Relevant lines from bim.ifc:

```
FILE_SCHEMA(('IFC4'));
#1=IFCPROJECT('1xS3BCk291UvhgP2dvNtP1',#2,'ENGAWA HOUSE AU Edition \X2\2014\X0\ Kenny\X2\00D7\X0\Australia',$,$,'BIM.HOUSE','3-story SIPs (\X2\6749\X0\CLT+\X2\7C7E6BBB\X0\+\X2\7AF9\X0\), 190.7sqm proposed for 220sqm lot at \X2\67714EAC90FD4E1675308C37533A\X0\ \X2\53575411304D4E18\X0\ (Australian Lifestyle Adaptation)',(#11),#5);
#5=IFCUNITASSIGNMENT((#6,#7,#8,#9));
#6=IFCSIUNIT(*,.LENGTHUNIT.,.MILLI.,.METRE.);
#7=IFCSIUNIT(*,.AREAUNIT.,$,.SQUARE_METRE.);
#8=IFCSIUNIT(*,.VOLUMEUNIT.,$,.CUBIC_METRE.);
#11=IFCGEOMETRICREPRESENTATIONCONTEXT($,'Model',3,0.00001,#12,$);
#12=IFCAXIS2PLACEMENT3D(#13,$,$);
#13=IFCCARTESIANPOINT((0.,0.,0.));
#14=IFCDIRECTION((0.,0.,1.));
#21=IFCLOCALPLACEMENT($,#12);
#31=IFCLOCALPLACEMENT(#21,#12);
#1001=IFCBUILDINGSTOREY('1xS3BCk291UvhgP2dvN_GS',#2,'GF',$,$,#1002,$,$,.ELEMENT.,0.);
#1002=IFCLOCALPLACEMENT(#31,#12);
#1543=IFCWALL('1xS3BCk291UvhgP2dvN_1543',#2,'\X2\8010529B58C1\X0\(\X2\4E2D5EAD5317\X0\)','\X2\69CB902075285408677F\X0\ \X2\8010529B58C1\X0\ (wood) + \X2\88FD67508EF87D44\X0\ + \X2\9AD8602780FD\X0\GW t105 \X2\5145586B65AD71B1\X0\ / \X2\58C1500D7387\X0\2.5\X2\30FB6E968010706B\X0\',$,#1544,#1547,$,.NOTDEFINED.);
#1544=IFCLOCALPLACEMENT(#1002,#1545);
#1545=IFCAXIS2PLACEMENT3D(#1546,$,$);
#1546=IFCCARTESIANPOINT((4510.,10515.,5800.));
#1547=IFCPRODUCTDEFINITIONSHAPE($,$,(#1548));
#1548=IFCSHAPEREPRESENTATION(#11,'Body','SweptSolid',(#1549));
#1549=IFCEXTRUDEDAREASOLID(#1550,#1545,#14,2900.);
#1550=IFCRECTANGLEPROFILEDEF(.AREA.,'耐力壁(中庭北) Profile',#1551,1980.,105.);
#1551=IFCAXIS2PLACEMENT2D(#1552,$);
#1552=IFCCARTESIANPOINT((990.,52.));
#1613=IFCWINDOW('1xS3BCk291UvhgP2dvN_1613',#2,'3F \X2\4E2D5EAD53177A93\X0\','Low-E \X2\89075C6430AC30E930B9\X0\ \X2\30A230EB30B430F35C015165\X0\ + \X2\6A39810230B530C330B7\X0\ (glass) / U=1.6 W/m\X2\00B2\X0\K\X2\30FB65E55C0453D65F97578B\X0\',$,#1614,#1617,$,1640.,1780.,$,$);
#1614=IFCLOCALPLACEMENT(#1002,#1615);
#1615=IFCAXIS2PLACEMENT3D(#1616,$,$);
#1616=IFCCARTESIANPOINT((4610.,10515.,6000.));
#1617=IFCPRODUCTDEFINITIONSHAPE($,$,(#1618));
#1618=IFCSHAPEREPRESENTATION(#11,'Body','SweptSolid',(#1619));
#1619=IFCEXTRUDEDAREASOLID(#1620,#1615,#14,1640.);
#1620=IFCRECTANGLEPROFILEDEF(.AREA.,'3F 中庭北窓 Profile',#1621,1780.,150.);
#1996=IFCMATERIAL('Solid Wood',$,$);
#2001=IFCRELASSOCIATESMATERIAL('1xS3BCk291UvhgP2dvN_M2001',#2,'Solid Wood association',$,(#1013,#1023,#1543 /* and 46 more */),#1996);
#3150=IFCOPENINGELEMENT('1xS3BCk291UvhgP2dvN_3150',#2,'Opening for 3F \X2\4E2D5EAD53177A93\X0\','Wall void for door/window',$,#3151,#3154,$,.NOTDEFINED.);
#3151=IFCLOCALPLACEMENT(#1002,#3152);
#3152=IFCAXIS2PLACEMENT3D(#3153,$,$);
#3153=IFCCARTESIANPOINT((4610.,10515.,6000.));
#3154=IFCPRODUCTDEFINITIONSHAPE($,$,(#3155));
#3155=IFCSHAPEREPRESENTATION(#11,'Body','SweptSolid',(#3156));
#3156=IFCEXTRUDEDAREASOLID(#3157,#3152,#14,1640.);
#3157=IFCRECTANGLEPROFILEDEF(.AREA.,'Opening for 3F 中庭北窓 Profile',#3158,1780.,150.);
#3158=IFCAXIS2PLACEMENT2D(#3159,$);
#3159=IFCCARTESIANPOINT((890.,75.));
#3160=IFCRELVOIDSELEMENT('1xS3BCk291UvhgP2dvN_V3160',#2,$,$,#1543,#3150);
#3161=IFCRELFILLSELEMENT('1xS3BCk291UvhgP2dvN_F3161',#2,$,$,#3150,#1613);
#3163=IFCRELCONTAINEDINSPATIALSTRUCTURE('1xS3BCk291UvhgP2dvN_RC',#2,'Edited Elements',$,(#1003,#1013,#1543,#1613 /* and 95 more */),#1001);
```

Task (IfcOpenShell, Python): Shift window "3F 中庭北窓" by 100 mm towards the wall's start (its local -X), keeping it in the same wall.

```python
import ifcopenshell
import ifcopenshell.api.geometry
import ifcopenshell.util.placement
import ifcopenshell.util.unit

model = ifcopenshell.open("bim.ifc")
unit_scale = ifcopenshell.util.unit.calculate_unit_scale(model)

window = model.by_guid("1xS3BCk291UvhgP2dvN_1613")
opening = window.FillsVoids[0].RelatingOpeningElement
wall = opening.VoidsElements[0].RelatingBuildingElement

wall_matrix = ifcopenshell.util.placement.get_local_placement(wall.ObjectPlacement)
shift = wall_matrix[:3, 0] * -0.1 / unit_scale
before = ifcopenshell.util.placement.get_local_placement(window.ObjectPlacement)[:3, 3].copy()

# The window is not placed relative to its opening, so move both.
for product in (opening, window):
    matrix = ifcopenshell.util.placement.get_local_placement(product.ObjectPlacement)
    matrix[:3, 3] += shift
    ifcopenshell.api.geometry.edit_object_placement(model, product=product, matrix=matrix, is_si=False)

after = ifcopenshell.util.placement.get_local_placement(window.ObjectPlacement)[:3, 3]
print("window moved by", (after - before).round(3) + 0.0)

model.write("bim-out.ifc")
```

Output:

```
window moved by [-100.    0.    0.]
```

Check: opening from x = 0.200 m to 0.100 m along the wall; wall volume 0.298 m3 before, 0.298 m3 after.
